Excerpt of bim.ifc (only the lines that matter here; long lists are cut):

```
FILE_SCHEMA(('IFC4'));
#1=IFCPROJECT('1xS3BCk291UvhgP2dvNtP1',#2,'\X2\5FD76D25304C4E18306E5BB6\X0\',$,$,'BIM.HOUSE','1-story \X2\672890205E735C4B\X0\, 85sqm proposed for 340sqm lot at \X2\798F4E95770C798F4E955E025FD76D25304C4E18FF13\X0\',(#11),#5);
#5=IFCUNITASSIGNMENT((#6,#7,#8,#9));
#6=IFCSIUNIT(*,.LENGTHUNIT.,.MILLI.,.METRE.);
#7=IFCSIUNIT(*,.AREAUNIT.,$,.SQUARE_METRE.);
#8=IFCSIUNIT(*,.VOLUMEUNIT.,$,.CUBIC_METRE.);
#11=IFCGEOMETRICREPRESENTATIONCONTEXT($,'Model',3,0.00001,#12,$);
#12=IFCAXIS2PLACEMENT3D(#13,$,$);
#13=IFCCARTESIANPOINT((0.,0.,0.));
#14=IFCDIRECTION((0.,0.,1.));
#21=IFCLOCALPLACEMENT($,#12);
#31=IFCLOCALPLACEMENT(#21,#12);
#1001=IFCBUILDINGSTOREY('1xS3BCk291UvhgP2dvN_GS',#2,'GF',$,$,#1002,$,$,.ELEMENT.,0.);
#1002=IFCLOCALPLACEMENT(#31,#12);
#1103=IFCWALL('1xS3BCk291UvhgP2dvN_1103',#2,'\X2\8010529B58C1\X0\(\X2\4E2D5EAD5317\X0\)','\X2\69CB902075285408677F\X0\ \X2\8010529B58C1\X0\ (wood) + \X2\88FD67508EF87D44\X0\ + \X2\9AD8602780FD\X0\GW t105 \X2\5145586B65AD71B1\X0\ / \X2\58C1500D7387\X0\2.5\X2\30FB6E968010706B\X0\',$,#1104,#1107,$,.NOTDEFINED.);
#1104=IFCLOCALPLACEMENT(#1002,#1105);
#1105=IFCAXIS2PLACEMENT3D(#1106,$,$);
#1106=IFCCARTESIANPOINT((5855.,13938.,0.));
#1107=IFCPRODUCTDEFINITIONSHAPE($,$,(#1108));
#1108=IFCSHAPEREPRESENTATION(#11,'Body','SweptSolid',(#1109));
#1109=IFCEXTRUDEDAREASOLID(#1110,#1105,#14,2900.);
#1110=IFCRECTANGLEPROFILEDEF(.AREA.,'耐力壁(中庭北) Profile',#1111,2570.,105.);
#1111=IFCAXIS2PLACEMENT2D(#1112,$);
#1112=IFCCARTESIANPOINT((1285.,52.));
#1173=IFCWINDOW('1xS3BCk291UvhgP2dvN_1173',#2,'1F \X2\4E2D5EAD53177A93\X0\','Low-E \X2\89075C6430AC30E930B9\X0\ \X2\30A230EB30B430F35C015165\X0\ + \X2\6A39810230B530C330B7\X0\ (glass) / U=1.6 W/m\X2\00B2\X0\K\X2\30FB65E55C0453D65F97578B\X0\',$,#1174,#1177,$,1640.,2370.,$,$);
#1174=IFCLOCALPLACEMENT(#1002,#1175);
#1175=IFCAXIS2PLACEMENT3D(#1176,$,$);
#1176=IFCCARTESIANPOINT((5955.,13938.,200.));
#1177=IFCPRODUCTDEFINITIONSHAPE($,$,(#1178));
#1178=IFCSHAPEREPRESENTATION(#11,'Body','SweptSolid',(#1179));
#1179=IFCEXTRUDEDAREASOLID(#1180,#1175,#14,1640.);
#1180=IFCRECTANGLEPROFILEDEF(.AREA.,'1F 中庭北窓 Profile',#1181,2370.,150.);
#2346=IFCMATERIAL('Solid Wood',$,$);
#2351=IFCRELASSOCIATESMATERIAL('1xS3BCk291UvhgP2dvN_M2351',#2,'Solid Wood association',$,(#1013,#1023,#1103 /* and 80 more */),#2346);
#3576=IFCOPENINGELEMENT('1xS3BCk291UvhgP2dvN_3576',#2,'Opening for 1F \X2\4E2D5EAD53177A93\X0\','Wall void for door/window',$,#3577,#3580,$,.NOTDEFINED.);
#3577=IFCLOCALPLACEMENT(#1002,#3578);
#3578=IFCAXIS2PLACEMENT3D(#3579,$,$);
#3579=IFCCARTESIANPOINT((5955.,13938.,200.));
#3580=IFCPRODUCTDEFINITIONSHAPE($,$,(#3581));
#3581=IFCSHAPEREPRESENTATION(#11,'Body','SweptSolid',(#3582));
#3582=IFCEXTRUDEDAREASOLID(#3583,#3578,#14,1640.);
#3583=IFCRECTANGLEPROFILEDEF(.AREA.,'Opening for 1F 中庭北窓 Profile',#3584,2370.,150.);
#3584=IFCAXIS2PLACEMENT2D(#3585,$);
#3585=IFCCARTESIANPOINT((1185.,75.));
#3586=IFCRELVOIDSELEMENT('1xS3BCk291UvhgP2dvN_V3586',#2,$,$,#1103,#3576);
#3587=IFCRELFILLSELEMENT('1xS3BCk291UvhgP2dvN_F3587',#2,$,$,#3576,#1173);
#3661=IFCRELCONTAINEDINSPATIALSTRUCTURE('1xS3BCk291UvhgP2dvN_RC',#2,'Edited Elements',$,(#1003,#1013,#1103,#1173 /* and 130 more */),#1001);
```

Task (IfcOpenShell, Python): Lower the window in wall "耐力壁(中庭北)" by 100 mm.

```python
import numpy as np
import ifcopenshell
import ifcopenshell.api.geometry
import ifcopenshell.util.placement
import ifcopenshell.util.unit

model = ifcopenshell.open("bim.ifc")
unit_scale = ifcopenshell.util.unit.calculate_unit_scale(model)

window = model.by_guid("1xS3BCk291UvhgP2dvN_1173")
opening = window.FillsVoids[0].RelatingOpeningElement
dz = -0.1 / unit_scale

shift = np.array([0.0, 0.0, dz])
# The window is not placed relative to its opening, so move both.
for product in (opening, window):
    matrix = ifcopenshell.util.placement.get_local_placement(product.ObjectPlacement)
    matrix[:3, 3] += shift
    ifcopenshell.api.geometry.edit_object_placement(model, product=product, matrix=matrix, is_si=False)

print(f"moved by {dz * unit_scale:+.3f} m")

model.write("bim-out.ifc")
```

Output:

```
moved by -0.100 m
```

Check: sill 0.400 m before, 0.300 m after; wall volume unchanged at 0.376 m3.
